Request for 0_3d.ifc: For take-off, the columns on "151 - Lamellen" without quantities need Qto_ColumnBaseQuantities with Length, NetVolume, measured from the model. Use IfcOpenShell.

First a look at what the model holds.

```python
import ifcopenshell
import ifcopenshell.util.element
import ifcopenshell.util.unit

model = ifcopenshell.open("0_3d.ifc")
print(model.schema)
for unit_type in ("LENGTHUNIT", "AREAUNIT", "VOLUMEUNIT"):
    print(unit_type, ifcopenshell.util.unit.calculate_unit_scale(model, unit_type))
storey = next(s for s in model.by_type("IfcBuildingStorey") if s.Name == "151 - Lamellen")
columns = [e for e in ifcopenshell.util.element.get_decomposition(storey) if e.is_a("IfcColumn")]
for e in sorted(columns, key=lambda e: e.id()):
    print(e.id(), e.is_a(), e.Name, list(ifcopenshell.util.element.get_psets(e, qtos_only=True)), sep=" | ")
```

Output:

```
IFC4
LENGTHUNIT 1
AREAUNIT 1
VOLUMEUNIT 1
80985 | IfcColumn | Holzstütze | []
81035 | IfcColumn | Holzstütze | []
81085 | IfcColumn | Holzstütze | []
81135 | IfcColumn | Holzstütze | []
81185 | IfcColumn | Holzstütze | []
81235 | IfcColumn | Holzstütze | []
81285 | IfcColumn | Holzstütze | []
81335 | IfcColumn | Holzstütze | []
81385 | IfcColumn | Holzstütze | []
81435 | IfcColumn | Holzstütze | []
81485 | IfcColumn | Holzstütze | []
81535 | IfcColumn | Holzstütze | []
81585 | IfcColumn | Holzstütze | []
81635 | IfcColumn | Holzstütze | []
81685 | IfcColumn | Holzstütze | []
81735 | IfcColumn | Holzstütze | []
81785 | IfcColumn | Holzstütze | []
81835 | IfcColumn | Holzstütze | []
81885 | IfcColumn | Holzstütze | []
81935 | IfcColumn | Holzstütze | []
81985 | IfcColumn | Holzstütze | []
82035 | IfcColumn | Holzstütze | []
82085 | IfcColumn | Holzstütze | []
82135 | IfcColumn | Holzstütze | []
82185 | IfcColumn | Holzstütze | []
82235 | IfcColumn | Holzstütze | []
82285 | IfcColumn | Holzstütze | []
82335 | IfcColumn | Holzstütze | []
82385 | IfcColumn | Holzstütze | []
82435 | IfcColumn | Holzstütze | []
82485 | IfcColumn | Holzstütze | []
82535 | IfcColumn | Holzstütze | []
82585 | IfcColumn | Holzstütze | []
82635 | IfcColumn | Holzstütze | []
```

```python
import ifcopenshell
import ifcopenshell.api.pset
import ifcopenshell.geom
import ifcopenshell.util.element
import ifcopenshell.util.shape
import ifcopenshell.util.unit

model = ifcopenshell.open("0_3d.ifc")
unit_scale = ifcopenshell.util.unit.calculate_unit_scale(model)
volume_scale = ifcopenshell.util.unit.calculate_unit_scale(model, "VOLUMEUNIT")
settings = ifcopenshell.geom.settings()

storey = next(s for s in model.by_type("IfcBuildingStorey") if s.Name == "151 - Lamellen")
columns = [e for e in ifcopenshell.util.element.get_decomposition(storey) if e.is_a("IfcColumn")]

for e in sorted(columns, key=lambda e: e.id()):
    if ifcopenshell.util.element.get_psets(e, qtos_only=True, should_inherit=False):
        continue
    # Geometry comes back in metres, in the element's own axes.
    shape = ifcopenshell.geom.create_shape(settings, e)
    values = {
        "Length": ifcopenshell.util.shape.get_z(shape.geometry) / unit_scale,
        "NetVolume": ifcopenshell.util.shape.get_volume(shape.geometry) / volume_scale,
    }
    qto = ifcopenshell.api.pset.add_qto(model, product=e, name="Qto_ColumnBaseQuantities")
    ifcopenshell.api.pset.edit_qto(model, qto=qto, properties=values)
    print(e.id(), {k: round(v, 3) for k, v in values.items()})

model.write("0_3d_rev.ifc")
```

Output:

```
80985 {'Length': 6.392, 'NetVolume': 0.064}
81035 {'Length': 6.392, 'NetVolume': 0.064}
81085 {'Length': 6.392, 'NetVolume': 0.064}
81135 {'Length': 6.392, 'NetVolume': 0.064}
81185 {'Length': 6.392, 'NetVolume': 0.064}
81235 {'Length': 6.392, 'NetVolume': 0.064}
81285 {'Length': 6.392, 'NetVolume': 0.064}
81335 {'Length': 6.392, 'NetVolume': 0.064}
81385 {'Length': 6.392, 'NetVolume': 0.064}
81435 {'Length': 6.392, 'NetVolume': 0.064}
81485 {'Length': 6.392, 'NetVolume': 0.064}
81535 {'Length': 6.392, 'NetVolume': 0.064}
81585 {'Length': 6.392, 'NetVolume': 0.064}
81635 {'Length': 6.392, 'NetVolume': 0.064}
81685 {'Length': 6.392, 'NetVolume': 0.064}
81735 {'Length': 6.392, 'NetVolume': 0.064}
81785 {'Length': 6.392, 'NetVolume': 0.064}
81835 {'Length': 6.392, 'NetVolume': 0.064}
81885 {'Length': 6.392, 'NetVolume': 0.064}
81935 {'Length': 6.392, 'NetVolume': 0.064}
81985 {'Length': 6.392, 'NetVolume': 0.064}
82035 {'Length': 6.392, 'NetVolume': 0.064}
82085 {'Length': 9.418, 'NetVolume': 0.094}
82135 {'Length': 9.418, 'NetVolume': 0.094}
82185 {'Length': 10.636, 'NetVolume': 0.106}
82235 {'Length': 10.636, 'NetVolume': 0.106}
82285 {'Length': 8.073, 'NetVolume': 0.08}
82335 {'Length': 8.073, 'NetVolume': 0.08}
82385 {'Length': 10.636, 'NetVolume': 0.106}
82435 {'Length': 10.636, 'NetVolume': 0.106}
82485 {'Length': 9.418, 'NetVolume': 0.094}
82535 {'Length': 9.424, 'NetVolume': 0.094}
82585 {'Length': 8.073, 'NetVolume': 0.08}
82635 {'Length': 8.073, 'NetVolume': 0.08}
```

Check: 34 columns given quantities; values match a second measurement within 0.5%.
